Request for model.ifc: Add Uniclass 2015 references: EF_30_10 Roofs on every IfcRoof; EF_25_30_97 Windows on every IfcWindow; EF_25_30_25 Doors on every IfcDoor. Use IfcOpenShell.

First a look at what the model holds.

```python
import ifcopenshell

model = ifcopenshell.open("model.ifc")
print(model.schema)
print("classifications:", [c.Name for c in model.by_type("IfcClassification")])
for ifc_class in ("IfcDoor", "IfcRoof", "IfcStair", "IfcWall", "IfcWindow"):
    print(ifc_class, len(model.by_type(ifc_class)))
```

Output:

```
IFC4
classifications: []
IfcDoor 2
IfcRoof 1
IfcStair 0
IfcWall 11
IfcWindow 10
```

```python
import ifcopenshell
import ifcopenshell.api.classification

model = ifcopenshell.open("model.ifc")

system = ifcopenshell.api.classification.add_classification(model, classification="Uniclass 2015")

codes = {
    "IfcRoof": ("EF_30_10", "Roofs"),
    "IfcWindow": ("EF_25_30_97", "Windows"),
    "IfcDoor": ("EF_25_30_25", "Doors"),
}
for ifc_class, (code, name) in codes.items():
    products = model.by_type(ifc_class)
    ifcopenshell.api.classification.add_reference(
        model, products=products, classification=system, identification=code, name=name
    )
    print(code, len(products))

model.write("model-out.ifc")
```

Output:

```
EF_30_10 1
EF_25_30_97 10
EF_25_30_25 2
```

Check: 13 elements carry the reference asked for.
